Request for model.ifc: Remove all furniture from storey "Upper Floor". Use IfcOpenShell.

First a look at what the model holds.

```python
import ifcopenshell
import ifcopenshell.util.element

model = ifcopenshell.open("model.ifc")
print(model.schema)
storey = next(s for s in model.by_type("IfcBuildingStorey") if s.Name == "Upper Floor")
furniture = [e for e in ifcopenshell.util.element.get_decomposition(storey) if e.is_a("IfcFurnishingElement")]
seen = {}
for e in furniture:
    element_type = ifcopenshell.util.element.get_type(e)
    name = element_type.Name if element_type not in (None, e) else None
    seen[name] = seen.get(name, 0) + 1
for name, count in sorted(seen.items(), key=str):
    print(count, "x", name)
```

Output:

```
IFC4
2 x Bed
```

```python
import ifcopenshell
import ifcopenshell.api.root
import ifcopenshell.util.element

model = ifcopenshell.open("model.ifc")

storey = next(s for s in model.by_type("IfcBuildingStorey") if s.Name == "Upper Floor")
furniture = [e for e in ifcopenshell.util.element.get_decomposition(storey) if e.is_a("IfcFurnishingElement")]

for e in furniture:
    ifcopenshell.api.root.remove_product(model, product=e)
print(len(furniture), "removed")

model.write("model_rev.ifc")
```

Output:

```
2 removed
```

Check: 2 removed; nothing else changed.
